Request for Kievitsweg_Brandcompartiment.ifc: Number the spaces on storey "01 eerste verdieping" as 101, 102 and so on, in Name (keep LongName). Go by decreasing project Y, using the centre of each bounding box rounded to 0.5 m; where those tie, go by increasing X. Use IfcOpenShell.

First a look at what the model holds.

```python
import ifcopenshell
import ifcopenshell.util.element
import ifcopenshell.util.placement

model = ifcopenshell.open("Kievitsweg_Brandcompartiment.ifc")
print(model.schema)
storey = next(s for s in model.by_type("IfcBuildingStorey") if s.Name == "01 eerste verdieping")
spaces = [e for e in ifcopenshell.util.element.get_decomposition(storey) if e.is_a("IfcSpace")]
for e in sorted(spaces, key=lambda e: e.id()):
    origin = ifcopenshell.util.placement.get_local_placement(e.ObjectPlacement)[:3, 3]
    print(e.id(), e.Name, e.LongName, origin.round(2) + 0.0, sep=" | ")
```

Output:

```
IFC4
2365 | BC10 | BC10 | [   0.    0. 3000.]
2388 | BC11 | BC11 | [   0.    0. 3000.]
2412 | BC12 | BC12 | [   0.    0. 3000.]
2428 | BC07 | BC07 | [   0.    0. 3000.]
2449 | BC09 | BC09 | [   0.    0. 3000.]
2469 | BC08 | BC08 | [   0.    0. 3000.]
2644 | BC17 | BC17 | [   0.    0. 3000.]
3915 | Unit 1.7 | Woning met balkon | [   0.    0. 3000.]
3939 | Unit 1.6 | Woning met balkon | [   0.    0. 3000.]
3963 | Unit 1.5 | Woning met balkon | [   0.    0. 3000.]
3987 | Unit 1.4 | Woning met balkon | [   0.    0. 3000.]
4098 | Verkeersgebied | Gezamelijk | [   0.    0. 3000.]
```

```python
import ifcopenshell
import ifcopenshell.geom
import ifcopenshell.util.element
import ifcopenshell.util.shape

model = ifcopenshell.open("Kievitsweg_Brandcompartiment.ifc")
settings = ifcopenshell.geom.settings()
settings.set("use-world-coords", True)


def centre(element):
    shape = ifcopenshell.geom.create_shape(settings, element)
    return ifcopenshell.util.shape.get_bbox_centroid(shape.geometry)


storey = next(s for s in model.by_type("IfcBuildingStorey") if s.Name == "01 eerste verdieping")
spaces = [e for e in ifcopenshell.util.element.get_decomposition(storey) if e.is_a("IfcSpace")]

# Insertion points can sit at a corner or the storey origin, so sort by the geometry (in metres).
centres = {e: centre(e) for e in spaces}
spaces.sort(key=lambda e: (-round(centres[e][1] / 0.5), centres[e][0]))

for i, e in enumerate(spaces, start=1):
    number = f"1{i:02d}"
    e.Name = number
    print(e.id(), number)

model.write("Kievitsweg_Brandcompartiment_edited.ifc")
```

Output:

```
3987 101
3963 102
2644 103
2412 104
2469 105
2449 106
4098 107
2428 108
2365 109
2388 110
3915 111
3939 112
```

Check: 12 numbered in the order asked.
